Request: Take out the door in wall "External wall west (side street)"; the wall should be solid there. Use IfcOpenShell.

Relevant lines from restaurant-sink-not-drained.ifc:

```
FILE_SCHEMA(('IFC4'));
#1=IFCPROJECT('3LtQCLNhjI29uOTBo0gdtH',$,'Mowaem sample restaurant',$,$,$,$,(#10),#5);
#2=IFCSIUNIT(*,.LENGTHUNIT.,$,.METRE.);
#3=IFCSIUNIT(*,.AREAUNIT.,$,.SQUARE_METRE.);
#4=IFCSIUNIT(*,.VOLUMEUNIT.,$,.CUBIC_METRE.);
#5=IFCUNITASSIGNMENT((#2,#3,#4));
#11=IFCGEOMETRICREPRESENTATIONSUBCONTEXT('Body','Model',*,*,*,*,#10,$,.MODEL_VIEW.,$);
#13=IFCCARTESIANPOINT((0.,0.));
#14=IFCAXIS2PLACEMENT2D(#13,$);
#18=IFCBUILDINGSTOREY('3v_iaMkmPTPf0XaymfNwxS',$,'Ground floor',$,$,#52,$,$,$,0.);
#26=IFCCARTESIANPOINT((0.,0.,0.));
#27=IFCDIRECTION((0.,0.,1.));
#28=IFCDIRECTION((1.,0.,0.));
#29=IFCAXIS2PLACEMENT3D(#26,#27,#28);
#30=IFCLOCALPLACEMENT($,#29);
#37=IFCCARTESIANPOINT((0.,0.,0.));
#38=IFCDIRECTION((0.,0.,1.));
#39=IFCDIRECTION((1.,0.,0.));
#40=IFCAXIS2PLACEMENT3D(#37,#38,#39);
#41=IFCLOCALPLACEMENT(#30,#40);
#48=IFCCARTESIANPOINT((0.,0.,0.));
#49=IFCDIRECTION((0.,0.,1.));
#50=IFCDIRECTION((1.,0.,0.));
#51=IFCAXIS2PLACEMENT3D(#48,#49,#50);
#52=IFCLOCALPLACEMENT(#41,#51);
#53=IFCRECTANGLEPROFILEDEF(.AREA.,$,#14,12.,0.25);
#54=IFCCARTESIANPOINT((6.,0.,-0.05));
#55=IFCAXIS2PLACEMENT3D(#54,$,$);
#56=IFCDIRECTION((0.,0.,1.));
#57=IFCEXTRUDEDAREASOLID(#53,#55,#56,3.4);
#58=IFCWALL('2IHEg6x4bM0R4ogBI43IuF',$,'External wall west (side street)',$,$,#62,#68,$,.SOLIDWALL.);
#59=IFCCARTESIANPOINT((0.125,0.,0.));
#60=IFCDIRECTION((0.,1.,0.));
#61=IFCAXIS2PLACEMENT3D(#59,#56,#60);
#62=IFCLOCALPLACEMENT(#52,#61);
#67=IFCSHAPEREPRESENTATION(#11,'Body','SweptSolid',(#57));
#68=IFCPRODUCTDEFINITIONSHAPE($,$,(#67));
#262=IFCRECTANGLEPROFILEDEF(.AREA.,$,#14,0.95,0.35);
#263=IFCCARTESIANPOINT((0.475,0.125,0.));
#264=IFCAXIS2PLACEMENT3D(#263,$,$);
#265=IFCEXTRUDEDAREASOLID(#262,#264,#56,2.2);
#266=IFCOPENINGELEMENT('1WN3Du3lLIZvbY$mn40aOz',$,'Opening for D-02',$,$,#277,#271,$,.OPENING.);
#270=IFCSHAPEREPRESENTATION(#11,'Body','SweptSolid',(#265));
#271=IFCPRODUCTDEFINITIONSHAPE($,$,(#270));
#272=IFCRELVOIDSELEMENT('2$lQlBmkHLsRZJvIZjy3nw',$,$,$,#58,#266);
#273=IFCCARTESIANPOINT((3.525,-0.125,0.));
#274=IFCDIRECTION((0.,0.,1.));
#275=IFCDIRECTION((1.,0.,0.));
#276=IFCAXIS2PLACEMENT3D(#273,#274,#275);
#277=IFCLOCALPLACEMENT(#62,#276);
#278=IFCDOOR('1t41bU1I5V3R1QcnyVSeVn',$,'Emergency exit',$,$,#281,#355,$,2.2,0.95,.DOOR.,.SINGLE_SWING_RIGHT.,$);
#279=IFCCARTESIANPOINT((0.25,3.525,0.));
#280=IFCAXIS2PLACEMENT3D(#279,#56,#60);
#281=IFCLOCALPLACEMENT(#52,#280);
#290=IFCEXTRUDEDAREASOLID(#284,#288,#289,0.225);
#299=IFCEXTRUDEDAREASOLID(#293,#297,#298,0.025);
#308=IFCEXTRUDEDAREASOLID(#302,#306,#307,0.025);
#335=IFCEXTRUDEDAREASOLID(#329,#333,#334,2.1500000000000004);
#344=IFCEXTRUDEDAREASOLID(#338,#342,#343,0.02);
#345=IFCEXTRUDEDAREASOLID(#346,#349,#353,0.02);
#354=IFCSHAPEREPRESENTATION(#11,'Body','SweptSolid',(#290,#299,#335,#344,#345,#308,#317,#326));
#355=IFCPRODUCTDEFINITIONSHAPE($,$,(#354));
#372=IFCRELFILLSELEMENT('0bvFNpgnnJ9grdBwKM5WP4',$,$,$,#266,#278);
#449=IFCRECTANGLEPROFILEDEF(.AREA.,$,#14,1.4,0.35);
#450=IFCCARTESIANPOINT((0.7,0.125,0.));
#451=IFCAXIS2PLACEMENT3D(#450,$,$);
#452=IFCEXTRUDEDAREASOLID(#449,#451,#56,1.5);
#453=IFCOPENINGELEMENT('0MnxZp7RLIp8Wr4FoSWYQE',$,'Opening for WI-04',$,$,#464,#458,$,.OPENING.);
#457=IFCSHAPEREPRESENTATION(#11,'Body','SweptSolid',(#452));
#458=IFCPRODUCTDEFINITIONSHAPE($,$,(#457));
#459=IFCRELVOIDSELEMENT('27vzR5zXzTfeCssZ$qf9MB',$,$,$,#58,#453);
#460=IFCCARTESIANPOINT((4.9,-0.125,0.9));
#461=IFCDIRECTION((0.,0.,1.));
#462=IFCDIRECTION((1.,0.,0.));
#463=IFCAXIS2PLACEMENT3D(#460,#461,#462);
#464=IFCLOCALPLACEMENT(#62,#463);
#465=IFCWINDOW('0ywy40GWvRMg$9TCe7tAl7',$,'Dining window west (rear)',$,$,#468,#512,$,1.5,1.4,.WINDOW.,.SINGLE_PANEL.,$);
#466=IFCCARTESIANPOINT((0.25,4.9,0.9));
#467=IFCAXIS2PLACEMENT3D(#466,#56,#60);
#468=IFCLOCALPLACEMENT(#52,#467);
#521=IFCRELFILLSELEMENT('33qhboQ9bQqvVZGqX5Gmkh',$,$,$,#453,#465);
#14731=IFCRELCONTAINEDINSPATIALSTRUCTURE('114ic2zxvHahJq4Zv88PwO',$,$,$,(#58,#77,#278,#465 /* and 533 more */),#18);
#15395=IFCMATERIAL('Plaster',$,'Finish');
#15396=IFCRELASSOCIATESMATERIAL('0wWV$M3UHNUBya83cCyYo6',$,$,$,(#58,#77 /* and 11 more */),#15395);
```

```python
import ifcopenshell
import ifcopenshell.api.feature
import ifcopenshell.api.root
import ifcopenshell.geom
import ifcopenshell.util.shape

model = ifcopenshell.open("restaurant-sink-not-drained.ifc")
settings = ifcopenshell.geom.settings()


def volume(element):
    """Net volume in cubic metres, openings subtracted."""
    shape = ifcopenshell.geom.create_shape(settings, element)
    return ifcopenshell.util.shape.get_volume(shape.geometry)


door = model.by_guid("1t41bU1I5V3R1QcnyVSeVn")
opening = door.FillsVoids[0].RelatingOpeningElement
wall = opening.VoidsElements[0].RelatingBuildingElement
before = volume(wall)

ifcopenshell.api.root.remove_product(model, product=door)
ifcopenshell.api.feature.remove_feature(model, feature=opening)

after = volume(wall)

print(f"wall volume {before:.3f} -> {after:.3f} m3")

model.write("restaurant-sink-not-drained-out.ifc")
```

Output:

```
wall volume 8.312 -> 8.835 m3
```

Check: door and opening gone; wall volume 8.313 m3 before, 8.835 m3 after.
